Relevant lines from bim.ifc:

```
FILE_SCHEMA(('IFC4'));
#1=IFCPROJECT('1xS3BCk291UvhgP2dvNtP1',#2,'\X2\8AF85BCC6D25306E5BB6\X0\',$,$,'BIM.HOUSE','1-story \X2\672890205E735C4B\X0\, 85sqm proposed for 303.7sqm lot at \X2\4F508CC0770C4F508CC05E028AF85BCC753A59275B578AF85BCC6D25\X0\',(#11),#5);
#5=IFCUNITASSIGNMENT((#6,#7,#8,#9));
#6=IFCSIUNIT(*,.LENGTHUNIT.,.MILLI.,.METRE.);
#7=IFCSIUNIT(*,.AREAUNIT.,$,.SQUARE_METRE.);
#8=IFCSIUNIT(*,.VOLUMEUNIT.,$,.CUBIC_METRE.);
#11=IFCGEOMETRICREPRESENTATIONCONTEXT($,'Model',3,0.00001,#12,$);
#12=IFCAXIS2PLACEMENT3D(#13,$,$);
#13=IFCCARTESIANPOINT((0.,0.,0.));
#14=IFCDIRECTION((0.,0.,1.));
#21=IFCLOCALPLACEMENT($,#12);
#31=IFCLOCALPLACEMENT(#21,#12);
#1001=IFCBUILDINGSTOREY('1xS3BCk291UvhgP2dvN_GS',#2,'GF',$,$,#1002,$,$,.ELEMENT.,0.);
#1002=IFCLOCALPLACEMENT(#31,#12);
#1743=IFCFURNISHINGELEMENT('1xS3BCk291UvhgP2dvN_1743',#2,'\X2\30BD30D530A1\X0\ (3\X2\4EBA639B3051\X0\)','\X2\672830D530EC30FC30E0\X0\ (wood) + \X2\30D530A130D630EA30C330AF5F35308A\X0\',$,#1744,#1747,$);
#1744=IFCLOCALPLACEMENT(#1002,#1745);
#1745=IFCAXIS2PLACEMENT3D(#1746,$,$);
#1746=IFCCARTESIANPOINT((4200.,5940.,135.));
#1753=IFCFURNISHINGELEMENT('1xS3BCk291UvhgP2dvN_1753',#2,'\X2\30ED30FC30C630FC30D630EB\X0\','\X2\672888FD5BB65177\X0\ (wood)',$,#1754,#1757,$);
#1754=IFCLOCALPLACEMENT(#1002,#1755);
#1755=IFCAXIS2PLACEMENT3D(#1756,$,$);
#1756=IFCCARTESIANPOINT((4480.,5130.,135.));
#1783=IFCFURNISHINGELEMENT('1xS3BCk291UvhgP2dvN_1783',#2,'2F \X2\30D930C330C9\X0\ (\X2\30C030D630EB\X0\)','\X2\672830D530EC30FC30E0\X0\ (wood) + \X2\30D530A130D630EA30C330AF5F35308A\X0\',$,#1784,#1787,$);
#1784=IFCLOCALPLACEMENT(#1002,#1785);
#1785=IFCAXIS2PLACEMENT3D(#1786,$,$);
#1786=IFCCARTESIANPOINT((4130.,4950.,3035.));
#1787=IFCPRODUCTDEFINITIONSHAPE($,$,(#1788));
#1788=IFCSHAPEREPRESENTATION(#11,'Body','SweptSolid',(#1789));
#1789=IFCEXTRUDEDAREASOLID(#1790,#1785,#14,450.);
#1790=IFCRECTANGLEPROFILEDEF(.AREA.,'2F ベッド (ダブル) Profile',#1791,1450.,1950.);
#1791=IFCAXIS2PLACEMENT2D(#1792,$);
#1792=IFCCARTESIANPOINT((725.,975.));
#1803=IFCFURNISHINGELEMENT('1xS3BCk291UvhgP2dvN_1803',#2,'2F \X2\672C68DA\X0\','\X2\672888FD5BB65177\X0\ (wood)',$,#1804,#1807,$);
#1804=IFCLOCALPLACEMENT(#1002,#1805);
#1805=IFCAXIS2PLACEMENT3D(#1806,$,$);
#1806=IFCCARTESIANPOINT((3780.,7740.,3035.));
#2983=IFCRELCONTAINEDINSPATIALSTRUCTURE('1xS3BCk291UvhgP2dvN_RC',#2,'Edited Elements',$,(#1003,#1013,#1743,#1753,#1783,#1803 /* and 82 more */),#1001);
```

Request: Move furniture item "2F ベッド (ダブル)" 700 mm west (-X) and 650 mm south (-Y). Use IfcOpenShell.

```python
import ifcopenshell
import ifcopenshell.api.geometry
import ifcopenshell.util.placement
import ifcopenshell.util.unit

model = ifcopenshell.open("bim.ifc")
unit_scale = ifcopenshell.util.unit.calculate_unit_scale(model)

item = model.by_id(1783)
matrix = ifcopenshell.util.placement.get_local_placement(item.ObjectPlacement)
matrix[0, 3] -= 0.7 / unit_scale
matrix[1, 3] -= 0.65 / unit_scale
ifcopenshell.api.geometry.edit_object_placement(model, product=item, matrix=matrix, is_si=False)

print(ifcopenshell.util.placement.get_local_placement(item.ObjectPlacement).round(3) + 0.0)

model.write("bim_rev.ifc")
```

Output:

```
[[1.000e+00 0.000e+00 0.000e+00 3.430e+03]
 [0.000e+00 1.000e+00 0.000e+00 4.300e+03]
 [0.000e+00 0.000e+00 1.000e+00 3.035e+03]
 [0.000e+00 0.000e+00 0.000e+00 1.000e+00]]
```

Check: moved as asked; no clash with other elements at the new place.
